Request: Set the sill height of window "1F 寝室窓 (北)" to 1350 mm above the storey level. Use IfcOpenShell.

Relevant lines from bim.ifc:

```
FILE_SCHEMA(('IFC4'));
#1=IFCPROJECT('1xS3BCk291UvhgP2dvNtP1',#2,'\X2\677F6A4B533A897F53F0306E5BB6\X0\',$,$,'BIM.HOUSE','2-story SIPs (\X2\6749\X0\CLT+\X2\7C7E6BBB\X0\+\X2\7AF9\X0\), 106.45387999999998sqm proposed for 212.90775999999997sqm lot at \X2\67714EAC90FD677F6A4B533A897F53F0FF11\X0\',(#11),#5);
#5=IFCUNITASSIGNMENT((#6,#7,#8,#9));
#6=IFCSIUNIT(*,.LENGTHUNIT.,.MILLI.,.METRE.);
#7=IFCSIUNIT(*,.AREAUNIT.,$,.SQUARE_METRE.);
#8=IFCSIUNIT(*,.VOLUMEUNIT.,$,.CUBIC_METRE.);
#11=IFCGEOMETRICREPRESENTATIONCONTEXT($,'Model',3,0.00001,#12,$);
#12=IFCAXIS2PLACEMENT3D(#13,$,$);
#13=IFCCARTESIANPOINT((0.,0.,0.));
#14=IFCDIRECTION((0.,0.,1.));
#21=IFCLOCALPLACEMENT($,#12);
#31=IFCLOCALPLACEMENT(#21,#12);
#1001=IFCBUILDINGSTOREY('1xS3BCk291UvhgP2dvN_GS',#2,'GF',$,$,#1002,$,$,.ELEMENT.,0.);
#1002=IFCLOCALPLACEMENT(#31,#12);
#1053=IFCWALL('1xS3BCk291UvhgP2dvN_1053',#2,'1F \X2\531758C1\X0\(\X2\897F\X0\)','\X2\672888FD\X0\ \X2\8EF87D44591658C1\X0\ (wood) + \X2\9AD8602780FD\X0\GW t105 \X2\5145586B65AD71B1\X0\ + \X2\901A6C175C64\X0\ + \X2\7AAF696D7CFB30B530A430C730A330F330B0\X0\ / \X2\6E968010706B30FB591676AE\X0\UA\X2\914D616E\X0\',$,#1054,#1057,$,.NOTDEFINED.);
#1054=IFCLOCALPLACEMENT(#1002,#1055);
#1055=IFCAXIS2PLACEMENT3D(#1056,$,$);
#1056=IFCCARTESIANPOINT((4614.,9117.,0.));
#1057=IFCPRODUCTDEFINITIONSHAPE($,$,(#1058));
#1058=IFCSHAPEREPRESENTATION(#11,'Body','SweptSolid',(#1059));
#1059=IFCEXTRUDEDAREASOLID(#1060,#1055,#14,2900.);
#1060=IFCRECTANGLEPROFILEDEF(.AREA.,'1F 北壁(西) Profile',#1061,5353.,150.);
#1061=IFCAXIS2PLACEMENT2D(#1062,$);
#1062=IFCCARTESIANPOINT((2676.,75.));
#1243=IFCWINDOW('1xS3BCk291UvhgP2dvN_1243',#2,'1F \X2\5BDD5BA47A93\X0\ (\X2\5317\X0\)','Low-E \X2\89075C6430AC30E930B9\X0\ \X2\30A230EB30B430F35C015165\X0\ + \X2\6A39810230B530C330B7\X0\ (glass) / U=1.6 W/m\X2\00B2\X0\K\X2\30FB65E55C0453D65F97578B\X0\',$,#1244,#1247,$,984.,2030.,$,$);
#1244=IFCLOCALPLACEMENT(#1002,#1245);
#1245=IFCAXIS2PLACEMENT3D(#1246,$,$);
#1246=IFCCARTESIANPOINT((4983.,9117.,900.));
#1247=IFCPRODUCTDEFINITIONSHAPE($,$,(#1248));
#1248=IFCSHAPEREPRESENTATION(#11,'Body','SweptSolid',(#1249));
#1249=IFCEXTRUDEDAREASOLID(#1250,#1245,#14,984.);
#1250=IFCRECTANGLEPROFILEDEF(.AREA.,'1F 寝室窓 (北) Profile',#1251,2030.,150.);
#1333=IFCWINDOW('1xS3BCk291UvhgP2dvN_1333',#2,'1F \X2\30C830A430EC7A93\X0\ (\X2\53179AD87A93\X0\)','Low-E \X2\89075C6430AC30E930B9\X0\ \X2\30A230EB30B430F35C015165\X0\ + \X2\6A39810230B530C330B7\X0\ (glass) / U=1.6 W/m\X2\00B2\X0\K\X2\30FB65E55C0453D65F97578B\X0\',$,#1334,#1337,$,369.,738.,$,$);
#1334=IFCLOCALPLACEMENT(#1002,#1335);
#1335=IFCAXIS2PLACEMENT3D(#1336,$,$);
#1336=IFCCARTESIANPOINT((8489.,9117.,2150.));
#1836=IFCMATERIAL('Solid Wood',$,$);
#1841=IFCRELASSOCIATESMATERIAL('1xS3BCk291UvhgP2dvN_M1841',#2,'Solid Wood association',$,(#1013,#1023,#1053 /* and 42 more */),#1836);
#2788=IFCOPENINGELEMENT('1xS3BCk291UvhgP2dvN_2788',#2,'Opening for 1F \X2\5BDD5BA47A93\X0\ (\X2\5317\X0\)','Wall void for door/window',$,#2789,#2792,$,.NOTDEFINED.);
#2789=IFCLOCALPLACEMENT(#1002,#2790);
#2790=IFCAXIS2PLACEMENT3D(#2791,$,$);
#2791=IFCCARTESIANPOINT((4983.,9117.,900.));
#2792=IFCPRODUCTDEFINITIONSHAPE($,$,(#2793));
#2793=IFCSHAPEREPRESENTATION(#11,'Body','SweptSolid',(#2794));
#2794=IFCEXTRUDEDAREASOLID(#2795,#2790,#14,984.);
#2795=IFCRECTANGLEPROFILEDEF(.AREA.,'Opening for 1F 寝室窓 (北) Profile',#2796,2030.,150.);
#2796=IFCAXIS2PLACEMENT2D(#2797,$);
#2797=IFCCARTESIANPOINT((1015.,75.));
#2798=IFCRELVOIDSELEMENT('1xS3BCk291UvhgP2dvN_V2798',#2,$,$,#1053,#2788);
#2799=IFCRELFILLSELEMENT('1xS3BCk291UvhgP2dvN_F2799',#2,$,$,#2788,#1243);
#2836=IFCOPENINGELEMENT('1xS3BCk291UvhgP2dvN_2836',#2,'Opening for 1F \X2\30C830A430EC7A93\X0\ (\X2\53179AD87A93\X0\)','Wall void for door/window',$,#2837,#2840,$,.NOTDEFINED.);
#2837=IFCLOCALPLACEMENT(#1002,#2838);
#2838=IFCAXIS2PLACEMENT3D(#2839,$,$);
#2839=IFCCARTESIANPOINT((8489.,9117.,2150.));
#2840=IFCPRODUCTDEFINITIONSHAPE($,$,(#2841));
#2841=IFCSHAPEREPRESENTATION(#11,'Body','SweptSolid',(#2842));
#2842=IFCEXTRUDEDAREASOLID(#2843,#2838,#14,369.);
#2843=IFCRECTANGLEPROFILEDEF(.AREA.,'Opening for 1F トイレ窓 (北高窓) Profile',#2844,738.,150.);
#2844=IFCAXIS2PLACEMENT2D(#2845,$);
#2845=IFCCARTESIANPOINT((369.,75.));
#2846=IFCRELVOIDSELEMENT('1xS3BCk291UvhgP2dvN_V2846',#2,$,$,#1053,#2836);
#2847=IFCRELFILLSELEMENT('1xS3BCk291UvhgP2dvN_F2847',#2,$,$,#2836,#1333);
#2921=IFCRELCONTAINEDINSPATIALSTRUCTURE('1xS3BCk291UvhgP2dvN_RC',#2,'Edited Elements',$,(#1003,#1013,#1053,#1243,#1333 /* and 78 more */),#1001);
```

```python
import numpy as np
import ifcopenshell
import ifcopenshell.api.geometry
import ifcopenshell.geom
import ifcopenshell.util.element
import ifcopenshell.util.placement
import ifcopenshell.util.shape
import ifcopenshell.util.unit

model = ifcopenshell.open("bim.ifc")
unit_scale = ifcopenshell.util.unit.calculate_unit_scale(model)

window = model.by_guid("1xS3BCk291UvhgP2dvN_1243")
opening = window.FillsVoids[0].RelatingOpeningElement
storey = ifcopenshell.util.element.get_container(window, ifc_class="IfcBuildingStorey")
level = ifcopenshell.util.placement.get_local_placement(storey.ObjectPlacement)[2, 3]

# The opening's origin need not be at the sill, so measure its lowest point.
shape = ifcopenshell.geom.create_shape(ifcopenshell.geom.settings(), opening)
bottom = ifcopenshell.util.shape.get_shape_bottom_elevation(shape, shape.geometry) / unit_scale
dz = level + 1.35 / unit_scale - bottom

shift = np.array([0.0, 0.0, dz])
# The window is not placed relative to its opening, so move both.
for product in (opening, window):
    matrix = ifcopenshell.util.placement.get_local_placement(product.ObjectPlacement)
    matrix[:3, 3] += shift
    ifcopenshell.api.geometry.edit_object_placement(model, product=product, matrix=matrix, is_si=False)

print(f"moved by {dz * unit_scale:+.3f} m")

model.write("bim_updated.ifc")
```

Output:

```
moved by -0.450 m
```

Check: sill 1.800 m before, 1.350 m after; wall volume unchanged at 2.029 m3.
